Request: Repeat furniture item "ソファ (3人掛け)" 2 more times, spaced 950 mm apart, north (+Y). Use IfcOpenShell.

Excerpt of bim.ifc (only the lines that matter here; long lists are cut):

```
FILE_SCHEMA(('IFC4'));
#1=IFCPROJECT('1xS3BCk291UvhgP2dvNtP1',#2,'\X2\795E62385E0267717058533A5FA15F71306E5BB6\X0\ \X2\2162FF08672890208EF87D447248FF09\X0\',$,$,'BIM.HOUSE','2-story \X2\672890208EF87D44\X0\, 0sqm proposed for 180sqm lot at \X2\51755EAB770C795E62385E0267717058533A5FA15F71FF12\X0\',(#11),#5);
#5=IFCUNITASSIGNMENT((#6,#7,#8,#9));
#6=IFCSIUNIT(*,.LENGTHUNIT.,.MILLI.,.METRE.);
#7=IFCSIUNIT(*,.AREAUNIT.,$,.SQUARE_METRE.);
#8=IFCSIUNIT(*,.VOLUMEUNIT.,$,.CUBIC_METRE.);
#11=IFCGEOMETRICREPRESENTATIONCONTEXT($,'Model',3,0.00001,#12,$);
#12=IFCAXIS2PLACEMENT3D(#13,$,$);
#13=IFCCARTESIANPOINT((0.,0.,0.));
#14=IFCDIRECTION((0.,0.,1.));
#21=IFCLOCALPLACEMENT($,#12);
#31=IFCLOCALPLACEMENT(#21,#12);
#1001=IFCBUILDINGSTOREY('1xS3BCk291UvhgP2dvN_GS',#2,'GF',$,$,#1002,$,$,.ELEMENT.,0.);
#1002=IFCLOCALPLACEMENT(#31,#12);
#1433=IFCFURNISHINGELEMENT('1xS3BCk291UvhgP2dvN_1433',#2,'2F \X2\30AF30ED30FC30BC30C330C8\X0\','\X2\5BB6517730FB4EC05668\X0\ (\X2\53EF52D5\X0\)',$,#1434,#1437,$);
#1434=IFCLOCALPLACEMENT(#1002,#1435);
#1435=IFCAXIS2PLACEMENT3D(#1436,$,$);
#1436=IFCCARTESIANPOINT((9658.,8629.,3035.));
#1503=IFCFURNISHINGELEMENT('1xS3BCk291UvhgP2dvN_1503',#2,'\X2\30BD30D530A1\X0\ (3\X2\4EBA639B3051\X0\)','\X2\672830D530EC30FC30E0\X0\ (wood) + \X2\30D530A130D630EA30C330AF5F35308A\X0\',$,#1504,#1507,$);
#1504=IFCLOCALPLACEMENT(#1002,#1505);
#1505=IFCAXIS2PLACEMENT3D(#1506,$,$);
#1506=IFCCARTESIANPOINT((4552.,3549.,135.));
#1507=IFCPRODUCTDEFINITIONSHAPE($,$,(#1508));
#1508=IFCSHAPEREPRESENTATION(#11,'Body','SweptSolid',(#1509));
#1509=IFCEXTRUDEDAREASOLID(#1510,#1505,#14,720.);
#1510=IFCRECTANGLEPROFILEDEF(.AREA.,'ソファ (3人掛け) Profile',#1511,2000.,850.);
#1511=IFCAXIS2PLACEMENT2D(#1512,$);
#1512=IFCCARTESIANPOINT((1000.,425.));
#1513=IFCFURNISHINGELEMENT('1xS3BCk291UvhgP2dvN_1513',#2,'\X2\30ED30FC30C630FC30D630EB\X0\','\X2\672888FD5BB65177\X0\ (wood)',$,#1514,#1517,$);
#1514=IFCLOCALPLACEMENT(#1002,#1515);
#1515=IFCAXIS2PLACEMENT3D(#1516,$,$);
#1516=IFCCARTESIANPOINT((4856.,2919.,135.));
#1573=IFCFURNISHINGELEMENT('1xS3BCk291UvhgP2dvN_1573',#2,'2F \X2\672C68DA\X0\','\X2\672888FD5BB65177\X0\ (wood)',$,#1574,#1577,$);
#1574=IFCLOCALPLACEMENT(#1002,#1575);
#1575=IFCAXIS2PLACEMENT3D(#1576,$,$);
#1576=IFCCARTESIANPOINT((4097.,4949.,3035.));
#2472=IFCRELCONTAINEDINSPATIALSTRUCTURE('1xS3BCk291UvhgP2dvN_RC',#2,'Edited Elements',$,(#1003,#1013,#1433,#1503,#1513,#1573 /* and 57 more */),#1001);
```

```python
import numpy as np
import ifcopenshell
import ifcopenshell.api.geometry
import ifcopenshell.api.root
import ifcopenshell.util.element
import ifcopenshell.util.placement
import ifcopenshell.util.unit

model = ifcopenshell.open("bim.ifc")
unit_scale = ifcopenshell.util.unit.calculate_unit_scale(model)


def reuse_history(source, copy):
    """copy_class also copies each property set's owner history, people and application; keep the originals."""
    for rel in copy.IsDefinedBy:
        if rel.is_a("IfcRelDefinesByProperties") and (history := rel.RelatingPropertyDefinition.OwnerHistory):
            rel.RelatingPropertyDefinition.OwnerHistory = source.OwnerHistory
            ifcopenshell.util.element.remove_deep2(model, history)


source = model.by_id(1503)
base = ifcopenshell.util.placement.get_local_placement(source.ObjectPlacement)
step = np.array([0.0, 1.0, 0.0]) * 0.95 / unit_scale

for i in range(1, 3):
    copy = ifcopenshell.api.root.copy_class(model, product=source)
    copy.Representation = ifcopenshell.util.element.copy_deep(
        model, source.Representation, exclude=["IfcGeometricRepresentationContext", "IfcRepresentationMap"]
    )
    reuse_history(source, copy)
    matrix = base.copy()
    matrix[:3, 3] += i * step
    print("added at", matrix[:3, 3].round(3) + 0.0)
    ifcopenshell.api.geometry.edit_object_placement(model, product=copy, matrix=matrix, is_si=False)

model.write("bim_edited.ifc")
```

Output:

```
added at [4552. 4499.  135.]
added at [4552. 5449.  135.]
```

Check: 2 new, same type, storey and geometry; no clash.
